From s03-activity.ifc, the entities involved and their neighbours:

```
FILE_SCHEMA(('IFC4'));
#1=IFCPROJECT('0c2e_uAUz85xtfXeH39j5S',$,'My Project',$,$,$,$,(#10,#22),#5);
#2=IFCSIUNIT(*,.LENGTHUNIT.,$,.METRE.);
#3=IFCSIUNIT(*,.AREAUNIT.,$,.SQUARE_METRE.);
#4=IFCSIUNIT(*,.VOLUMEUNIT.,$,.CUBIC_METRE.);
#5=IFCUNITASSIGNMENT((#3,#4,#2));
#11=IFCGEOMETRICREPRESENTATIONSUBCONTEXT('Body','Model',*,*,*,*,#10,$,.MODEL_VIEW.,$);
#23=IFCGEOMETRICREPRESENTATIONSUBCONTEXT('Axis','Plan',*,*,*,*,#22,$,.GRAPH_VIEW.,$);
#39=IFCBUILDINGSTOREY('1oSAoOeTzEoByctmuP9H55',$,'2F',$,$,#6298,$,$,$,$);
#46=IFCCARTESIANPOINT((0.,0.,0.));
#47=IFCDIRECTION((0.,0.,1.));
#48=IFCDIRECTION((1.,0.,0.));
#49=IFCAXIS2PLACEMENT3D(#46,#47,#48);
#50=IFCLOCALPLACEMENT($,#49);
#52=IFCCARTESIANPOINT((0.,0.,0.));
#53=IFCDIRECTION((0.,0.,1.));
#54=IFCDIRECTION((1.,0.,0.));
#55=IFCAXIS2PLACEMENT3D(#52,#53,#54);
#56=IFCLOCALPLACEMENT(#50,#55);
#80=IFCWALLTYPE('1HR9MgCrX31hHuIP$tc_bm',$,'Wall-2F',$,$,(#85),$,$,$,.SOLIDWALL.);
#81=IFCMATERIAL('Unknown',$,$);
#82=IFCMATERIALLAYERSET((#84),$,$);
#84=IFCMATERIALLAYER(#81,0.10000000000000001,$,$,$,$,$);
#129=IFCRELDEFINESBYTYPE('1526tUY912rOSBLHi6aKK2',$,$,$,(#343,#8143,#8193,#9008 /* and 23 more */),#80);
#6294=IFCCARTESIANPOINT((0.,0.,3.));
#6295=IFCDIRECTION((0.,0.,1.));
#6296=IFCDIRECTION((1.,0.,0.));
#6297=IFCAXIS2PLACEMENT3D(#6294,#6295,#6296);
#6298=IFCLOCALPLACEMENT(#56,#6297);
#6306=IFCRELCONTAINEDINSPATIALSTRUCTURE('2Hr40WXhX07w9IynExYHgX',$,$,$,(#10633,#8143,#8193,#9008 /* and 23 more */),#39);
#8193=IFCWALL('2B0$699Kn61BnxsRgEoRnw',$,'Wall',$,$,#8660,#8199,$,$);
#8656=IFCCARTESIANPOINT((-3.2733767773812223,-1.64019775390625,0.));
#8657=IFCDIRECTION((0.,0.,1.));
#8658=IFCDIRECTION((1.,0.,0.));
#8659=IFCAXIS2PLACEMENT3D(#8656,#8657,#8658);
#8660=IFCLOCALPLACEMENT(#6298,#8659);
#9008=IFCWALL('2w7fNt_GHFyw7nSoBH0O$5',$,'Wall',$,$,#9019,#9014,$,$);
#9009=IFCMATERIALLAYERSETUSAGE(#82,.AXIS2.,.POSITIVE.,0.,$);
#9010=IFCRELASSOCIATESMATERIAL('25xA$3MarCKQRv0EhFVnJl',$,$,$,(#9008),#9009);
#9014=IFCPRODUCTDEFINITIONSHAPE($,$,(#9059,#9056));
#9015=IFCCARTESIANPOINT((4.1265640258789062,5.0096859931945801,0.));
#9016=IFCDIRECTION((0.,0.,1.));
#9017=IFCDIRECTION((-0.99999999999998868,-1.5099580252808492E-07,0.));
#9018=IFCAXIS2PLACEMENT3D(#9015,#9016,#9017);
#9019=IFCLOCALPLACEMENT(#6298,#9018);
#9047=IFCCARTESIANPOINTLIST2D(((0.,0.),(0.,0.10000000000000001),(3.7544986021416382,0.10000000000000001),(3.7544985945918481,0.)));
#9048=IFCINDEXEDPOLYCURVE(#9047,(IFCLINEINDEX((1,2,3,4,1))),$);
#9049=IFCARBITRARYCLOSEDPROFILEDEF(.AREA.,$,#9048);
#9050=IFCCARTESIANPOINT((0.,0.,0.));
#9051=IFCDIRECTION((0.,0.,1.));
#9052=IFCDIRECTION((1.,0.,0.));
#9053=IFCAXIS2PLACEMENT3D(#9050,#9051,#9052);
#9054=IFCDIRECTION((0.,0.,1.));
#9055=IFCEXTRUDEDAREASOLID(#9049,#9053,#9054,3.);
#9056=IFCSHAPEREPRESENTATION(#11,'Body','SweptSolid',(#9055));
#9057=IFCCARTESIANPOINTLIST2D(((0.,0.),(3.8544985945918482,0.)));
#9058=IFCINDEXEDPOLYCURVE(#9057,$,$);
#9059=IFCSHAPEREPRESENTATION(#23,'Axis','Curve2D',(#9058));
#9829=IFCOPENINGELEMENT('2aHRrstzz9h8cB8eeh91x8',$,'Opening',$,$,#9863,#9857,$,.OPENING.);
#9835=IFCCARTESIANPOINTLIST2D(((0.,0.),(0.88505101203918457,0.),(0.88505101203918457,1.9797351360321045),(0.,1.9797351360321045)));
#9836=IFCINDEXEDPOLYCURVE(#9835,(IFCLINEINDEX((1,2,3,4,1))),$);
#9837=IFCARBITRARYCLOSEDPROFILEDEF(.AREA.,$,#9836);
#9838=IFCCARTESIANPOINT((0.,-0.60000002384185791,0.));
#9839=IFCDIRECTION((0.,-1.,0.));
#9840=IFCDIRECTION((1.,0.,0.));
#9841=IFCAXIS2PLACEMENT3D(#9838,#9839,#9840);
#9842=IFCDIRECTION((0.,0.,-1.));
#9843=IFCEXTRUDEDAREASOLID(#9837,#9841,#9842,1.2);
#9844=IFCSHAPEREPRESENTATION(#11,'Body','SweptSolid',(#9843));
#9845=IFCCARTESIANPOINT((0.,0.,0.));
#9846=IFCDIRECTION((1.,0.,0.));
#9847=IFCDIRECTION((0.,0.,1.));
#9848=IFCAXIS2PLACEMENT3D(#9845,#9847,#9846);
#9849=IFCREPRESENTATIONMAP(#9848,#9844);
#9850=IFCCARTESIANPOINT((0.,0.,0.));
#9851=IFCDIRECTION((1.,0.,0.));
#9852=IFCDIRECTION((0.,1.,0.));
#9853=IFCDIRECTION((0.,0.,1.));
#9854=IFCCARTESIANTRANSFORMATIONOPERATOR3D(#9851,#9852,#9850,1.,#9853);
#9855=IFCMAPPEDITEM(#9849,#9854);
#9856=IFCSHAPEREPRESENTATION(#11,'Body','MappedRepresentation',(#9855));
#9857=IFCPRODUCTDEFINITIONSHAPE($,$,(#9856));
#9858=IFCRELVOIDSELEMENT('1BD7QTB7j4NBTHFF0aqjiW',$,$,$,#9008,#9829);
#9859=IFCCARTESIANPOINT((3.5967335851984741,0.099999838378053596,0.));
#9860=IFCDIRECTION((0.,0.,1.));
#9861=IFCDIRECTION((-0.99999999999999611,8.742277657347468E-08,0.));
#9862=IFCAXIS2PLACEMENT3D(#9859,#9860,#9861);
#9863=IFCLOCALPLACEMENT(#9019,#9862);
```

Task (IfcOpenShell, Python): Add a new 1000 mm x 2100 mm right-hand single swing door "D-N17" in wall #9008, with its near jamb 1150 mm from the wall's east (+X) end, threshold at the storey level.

```python
import numpy as np
import ifcopenshell
import ifcopenshell.api.feature
import ifcopenshell.api.geometry
import ifcopenshell.api.root
import ifcopenshell.api.spatial
import ifcopenshell.geom
import ifcopenshell.util.element
import ifcopenshell.util.placement
import ifcopenshell.util.representation
import ifcopenshell.util.shape
import ifcopenshell.util.unit

model = ifcopenshell.open("s03-activity.ifc")
unit_scale = ifcopenshell.util.unit.calculate_unit_scale(model)
settings = ifcopenshell.geom.settings()


def volume(element):
    """Net volume in cubic metres, openings subtracted."""
    shape = ifcopenshell.geom.create_shape(settings, element)
    return ifcopenshell.util.shape.get_volume(shape.geometry)


wall = model.by_guid("2w7fNt_GHFyw7nSoBH0O$5")
storey = ifcopenshell.util.element.get_container(wall, ifc_class="IfcBuildingStorey")
context = ifcopenshell.util.representation.get_context(model, "Model", "Body", "MODEL_VIEW")
before = volume(wall)

width, height, from_end, sill = 1, 2.1, 1.15, 0.0  # metres

# The wall runs along its own X axis, and the end named is its -X end.
wall_shape = ifcopenshell.geom.create_shape(settings, wall)
x, y, z = ifcopenshell.util.shape.get_vertices(wall_shape.geometry).T
start = x.min() + from_end
face, thickness = float(y.min()), float(y.max() - y.min())
wall_matrix = ifcopenshell.util.placement.get_local_placement(wall.ObjectPlacement)
level = ifcopenshell.util.placement.get_local_placement(storey.ObjectPlacement)[2, 3]


def in_wall(x, y):
    """Placement at x, y metres in the wall's axes, at sill height."""
    matrix = wall_matrix.copy()
    matrix[:, 3] = wall_matrix @ np.array([x / unit_scale, y / unit_scale, 0.0, 1.0])
    matrix[2, 3] = level + sill / unit_scale
    return matrix


# Opening: a box that overshoots both wall faces by 50 mm.
opening = ifcopenshell.api.root.create_entity(model, ifc_class="IfcOpeningElement", predefined_type="OPENING")
box = ifcopenshell.api.geometry.add_wall_representation(
    model, context=context, length=width, height=height, thickness=thickness + 0.1
)
ifcopenshell.api.geometry.assign_representation(model, product=opening, representation=box)
ifcopenshell.api.geometry.edit_object_placement(model, product=opening, matrix=in_wall(start, face - 0.05), is_si=False)
ifcopenshell.api.feature.add_feature(model, feature=opening, element=wall)

door = ifcopenshell.api.root.create_entity(model, ifc_class="IfcDoor", name="D-N17", predefined_type="DOOR")
door.OverallWidth, door.OverallHeight = width / unit_scale, height / unit_scale
door.OperationType = "SINGLE_SWING_RIGHT"
body = ifcopenshell.api.geometry.add_door_representation(
    model,
    context=context,
    overall_width=door.OverallWidth,
    overall_height=door.OverallHeight,
    operation_type="SINGLE_SWING_RIGHT",
    lining_properties={"LiningDepth": thickness / unit_scale, "ThresholdDepth": thickness / unit_scale},
)
ifcopenshell.api.geometry.assign_representation(model, product=door, representation=body)
ifcopenshell.api.spatial.assign_container(model, products=[door], relating_structure=storey)
ifcopenshell.api.feature.add_filling(model, opening=opening, element=door)

# The lining spans the wall, so the door starts at the wall face.
ifcopenshell.api.geometry.edit_object_placement(model, product=door, matrix=in_wall(start, face), is_si=False)

after = volume(wall)

print(f"wall volume {before:.3f} -> {after:.3f} m3")

model.write("s03-activity-out.ifc")
```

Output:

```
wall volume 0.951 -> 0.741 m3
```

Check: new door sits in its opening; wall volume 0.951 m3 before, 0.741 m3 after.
